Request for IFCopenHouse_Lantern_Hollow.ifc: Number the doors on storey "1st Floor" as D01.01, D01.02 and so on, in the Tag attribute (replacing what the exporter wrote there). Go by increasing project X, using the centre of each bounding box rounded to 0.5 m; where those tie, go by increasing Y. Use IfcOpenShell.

First a look at what the model holds.

```python
import ifcopenshell
import ifcopenshell.util.element
import ifcopenshell.util.placement

model = ifcopenshell.open("IFCopenHouse_Lantern_Hollow.ifc")
print(model.schema)
storey = next(s for s in model.by_type("IfcBuildingStorey") if s.Name == "1st Floor")
doors = [e for e in ifcopenshell.util.element.get_decomposition(storey) if e.is_a("IfcDoor")]
for e in sorted(doors, key=lambda e: e.id()):
    origin = ifcopenshell.util.placement.get_local_placement(e.ObjectPlacement)[:3, 3]
    print(e.id(), e.Tag, e.Name, origin.round(2) + 0.0, sep=" | ")
```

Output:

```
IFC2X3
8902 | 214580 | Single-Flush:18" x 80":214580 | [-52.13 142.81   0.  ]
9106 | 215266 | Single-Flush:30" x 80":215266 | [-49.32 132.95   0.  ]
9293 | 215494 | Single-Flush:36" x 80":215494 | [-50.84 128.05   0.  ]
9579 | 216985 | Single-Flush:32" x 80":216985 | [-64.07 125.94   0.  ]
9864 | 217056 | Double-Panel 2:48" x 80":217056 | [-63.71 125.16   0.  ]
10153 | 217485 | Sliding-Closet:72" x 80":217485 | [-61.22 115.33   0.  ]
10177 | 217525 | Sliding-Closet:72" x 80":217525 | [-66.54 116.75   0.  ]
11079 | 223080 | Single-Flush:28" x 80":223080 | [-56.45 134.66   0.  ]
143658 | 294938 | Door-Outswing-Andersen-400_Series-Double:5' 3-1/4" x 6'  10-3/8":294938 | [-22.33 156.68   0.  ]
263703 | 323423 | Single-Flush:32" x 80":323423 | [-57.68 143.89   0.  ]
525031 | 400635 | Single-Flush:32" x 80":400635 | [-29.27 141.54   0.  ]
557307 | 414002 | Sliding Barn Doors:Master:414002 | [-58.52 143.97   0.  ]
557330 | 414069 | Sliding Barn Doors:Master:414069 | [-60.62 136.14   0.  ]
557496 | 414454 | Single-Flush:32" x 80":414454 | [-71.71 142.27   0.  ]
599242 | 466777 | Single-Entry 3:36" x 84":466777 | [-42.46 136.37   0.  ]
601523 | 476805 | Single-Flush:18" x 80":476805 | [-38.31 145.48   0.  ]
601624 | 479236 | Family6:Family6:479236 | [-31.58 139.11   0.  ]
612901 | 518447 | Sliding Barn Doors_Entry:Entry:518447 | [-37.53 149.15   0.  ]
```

```python
import ifcopenshell
import ifcopenshell.geom
import ifcopenshell.util.element
import ifcopenshell.util.shape

model = ifcopenshell.open("IFCopenHouse_Lantern_Hollow.ifc")
settings = ifcopenshell.geom.settings()
settings.set("use-world-coords", True)


def centre(element):
    shape = ifcopenshell.geom.create_shape(settings, element)
    return ifcopenshell.util.shape.get_bbox_centroid(shape.geometry)


storey = next(s for s in model.by_type("IfcBuildingStorey") if s.Name == "1st Floor")
doors = [e for e in ifcopenshell.util.element.get_decomposition(storey) if e.is_a("IfcDoor")]

# Insertion points can sit at a corner or the storey origin, so sort by the geometry (in metres).
centres = {e: centre(e) for e in doors}
doors.sort(key=lambda e: (round(centres[e][0] / 0.5), centres[e][1]))

for i, e in enumerate(doors, start=1):
    number = f"D01.{i:02d}"
    e.Tag = number
    print(e.id(), number)

model.write("IFCopenHouse_Lantern_Hollow_edited.ifc")
```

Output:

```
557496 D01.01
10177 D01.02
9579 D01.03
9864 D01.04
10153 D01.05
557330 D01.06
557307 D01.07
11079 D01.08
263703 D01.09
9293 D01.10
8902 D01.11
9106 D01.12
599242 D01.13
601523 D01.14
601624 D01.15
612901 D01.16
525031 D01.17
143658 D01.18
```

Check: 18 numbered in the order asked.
